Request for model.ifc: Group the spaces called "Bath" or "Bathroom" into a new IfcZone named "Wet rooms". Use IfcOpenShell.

First a look at what the model holds.

```python
import ifcopenshell

model = ifcopenshell.open("model.ifc")
print(model.schema)
seen = {}
for space in model.by_type("IfcSpace"):
    seen[space.LongName] = seen.get(space.LongName, 0) + 1
for name, count in sorted(seen.items(), key=str):
    print(count, "x", name)
print("zones:", [z.Name for z in model.by_type("IfcZone")][:20])
```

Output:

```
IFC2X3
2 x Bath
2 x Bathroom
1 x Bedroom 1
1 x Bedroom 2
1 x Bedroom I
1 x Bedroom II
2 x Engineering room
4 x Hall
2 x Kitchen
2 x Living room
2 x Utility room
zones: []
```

```python
import ifcopenshell
import ifcopenshell.api.group
import ifcopenshell.api.root

model = ifcopenshell.open("model.ifc")

names = {"Bath", "Bathroom"}
spaces = [s for s in model.by_type("IfcSpace") if s.LongName in names]

zone = ifcopenshell.api.root.create_entity(model, ifc_class="IfcZone", name="Wet rooms")
ifcopenshell.api.group.assign_group(model, products=spaces, group=zone)
print(len(spaces), "spaces in", zone.Name)

model.write("model_rev.ifc")
```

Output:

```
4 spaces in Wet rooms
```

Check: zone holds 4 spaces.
